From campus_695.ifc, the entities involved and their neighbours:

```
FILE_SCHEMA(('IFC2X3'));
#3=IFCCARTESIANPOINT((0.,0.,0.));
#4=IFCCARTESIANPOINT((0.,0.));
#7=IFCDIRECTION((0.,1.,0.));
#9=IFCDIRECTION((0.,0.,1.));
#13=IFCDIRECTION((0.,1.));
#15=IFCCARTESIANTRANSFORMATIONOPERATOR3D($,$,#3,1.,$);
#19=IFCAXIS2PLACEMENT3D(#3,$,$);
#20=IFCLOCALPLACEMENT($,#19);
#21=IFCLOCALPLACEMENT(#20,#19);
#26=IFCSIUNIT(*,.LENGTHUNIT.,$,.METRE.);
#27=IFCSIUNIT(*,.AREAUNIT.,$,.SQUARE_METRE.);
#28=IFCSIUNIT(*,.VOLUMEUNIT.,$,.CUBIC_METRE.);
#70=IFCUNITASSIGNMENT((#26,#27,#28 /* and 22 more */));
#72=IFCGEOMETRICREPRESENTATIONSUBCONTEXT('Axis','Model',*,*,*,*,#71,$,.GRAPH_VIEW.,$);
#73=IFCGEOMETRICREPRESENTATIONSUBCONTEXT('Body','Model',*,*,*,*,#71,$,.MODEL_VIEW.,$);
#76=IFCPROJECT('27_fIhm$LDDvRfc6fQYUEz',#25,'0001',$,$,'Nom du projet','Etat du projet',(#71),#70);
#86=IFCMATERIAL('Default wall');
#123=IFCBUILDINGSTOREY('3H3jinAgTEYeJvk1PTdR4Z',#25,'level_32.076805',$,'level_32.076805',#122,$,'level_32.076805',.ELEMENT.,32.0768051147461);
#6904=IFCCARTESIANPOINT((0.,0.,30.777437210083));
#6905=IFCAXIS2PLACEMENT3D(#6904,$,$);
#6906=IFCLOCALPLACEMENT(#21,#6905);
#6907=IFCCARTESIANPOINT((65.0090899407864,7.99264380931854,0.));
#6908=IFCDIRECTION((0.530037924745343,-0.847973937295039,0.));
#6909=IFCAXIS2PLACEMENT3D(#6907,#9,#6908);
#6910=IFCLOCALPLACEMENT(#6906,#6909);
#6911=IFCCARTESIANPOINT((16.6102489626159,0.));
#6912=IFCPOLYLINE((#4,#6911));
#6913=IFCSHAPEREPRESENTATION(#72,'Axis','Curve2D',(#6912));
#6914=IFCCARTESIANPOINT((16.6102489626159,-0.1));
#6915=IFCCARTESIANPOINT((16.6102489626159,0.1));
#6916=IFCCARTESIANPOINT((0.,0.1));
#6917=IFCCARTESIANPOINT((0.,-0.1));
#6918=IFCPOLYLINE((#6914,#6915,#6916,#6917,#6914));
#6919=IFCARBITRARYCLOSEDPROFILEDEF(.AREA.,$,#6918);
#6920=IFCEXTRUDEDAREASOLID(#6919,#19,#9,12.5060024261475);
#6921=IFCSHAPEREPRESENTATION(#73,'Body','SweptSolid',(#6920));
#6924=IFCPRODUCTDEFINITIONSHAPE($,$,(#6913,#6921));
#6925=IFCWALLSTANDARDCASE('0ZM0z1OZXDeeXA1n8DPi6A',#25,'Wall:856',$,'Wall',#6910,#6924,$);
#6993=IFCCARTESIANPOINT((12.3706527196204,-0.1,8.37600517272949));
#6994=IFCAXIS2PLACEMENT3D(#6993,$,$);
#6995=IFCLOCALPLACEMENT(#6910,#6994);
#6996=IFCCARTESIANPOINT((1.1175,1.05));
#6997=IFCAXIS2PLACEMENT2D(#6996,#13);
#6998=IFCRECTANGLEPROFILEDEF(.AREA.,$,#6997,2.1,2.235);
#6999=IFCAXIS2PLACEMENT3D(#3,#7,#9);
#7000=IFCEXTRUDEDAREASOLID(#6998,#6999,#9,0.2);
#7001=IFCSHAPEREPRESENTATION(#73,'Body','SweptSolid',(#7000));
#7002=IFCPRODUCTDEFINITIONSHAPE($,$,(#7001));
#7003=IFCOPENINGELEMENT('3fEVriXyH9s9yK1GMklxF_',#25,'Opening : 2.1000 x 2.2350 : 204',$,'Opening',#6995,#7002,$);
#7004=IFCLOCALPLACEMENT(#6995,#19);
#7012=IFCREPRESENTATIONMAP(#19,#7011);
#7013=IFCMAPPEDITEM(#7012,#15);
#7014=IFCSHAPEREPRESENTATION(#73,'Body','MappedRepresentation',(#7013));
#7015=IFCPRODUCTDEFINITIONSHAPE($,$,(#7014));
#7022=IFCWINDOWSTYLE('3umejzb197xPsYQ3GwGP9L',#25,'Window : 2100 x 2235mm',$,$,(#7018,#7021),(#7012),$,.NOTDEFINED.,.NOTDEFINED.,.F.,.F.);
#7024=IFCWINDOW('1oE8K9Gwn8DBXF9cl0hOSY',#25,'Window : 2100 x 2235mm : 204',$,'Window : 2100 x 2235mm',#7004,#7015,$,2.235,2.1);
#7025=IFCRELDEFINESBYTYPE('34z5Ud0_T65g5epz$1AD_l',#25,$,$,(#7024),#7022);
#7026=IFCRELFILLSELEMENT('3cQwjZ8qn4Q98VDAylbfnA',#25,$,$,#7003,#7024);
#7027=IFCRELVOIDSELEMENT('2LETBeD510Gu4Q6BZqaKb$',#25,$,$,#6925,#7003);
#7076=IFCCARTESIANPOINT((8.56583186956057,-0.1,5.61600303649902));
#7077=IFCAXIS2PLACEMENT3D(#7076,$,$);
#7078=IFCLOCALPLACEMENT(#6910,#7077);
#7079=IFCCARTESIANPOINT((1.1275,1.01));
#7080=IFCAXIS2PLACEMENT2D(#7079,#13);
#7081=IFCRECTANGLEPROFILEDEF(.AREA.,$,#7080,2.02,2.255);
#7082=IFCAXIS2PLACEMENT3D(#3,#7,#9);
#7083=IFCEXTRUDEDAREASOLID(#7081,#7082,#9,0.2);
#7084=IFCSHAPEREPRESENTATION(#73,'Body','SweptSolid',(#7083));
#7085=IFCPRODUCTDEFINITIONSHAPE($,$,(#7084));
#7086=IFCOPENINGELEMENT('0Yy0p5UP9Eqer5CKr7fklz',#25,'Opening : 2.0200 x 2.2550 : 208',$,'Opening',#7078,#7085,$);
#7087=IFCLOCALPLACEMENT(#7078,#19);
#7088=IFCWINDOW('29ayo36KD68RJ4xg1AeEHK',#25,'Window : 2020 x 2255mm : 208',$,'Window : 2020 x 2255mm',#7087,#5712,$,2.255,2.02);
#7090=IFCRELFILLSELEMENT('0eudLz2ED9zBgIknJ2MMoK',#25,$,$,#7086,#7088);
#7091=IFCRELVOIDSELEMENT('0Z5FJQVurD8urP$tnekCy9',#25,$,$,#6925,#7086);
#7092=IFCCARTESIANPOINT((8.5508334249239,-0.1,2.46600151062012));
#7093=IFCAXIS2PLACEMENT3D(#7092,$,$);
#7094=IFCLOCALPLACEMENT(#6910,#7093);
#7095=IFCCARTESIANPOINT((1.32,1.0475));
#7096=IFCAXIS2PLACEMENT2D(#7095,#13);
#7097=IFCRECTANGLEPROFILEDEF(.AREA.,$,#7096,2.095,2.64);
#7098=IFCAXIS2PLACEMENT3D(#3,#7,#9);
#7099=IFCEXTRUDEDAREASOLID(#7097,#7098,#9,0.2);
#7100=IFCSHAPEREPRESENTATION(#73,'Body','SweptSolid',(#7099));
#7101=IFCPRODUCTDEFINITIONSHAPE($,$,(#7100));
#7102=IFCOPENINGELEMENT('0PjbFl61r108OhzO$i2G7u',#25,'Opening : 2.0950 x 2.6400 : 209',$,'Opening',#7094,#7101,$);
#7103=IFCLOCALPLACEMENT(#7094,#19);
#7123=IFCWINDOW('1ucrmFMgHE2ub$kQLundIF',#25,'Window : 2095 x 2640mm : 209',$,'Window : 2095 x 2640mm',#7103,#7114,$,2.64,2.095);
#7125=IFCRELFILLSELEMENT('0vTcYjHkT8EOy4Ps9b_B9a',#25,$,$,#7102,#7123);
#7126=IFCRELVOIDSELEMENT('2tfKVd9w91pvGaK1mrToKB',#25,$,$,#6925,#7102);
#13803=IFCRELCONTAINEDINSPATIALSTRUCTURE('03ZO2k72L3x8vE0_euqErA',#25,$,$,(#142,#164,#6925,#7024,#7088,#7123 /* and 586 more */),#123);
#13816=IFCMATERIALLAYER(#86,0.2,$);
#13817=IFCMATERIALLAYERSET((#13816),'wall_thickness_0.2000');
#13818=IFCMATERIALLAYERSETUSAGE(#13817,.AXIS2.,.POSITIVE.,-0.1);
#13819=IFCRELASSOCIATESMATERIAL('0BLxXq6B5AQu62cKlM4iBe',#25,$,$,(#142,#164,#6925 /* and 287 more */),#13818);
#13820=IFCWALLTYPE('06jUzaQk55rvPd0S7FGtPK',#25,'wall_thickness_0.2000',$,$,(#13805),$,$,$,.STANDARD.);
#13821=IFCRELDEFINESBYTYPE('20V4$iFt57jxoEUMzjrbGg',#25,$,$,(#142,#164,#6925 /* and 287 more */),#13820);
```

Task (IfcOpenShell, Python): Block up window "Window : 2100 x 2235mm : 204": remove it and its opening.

```python
import ifcopenshell
import ifcopenshell.api.feature
import ifcopenshell.api.root
import ifcopenshell.geom
import ifcopenshell.util.shape

model = ifcopenshell.open("campus_695.ifc")
settings = ifcopenshell.geom.settings()


def volume(element):
    """Net volume in cubic metres, openings subtracted."""
    shape = ifcopenshell.geom.create_shape(settings, element)
    return ifcopenshell.util.shape.get_volume(shape.geometry)


window = model.by_guid("1oE8K9Gwn8DBXF9cl0hOSY")
opening = window.FillsVoids[0].RelatingOpeningElement
wall = opening.VoidsElements[0].RelatingBuildingElement
before = volume(wall)

ifcopenshell.api.root.remove_product(model, product=window)
ifcopenshell.api.feature.remove_feature(model, feature=opening)

after = volume(wall)

print(f"wall volume {before:.3f} -> {after:.3f} m3")

model.write("campus_695_updated.ifc")
```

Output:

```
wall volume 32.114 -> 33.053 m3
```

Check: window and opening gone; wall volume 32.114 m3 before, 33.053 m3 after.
